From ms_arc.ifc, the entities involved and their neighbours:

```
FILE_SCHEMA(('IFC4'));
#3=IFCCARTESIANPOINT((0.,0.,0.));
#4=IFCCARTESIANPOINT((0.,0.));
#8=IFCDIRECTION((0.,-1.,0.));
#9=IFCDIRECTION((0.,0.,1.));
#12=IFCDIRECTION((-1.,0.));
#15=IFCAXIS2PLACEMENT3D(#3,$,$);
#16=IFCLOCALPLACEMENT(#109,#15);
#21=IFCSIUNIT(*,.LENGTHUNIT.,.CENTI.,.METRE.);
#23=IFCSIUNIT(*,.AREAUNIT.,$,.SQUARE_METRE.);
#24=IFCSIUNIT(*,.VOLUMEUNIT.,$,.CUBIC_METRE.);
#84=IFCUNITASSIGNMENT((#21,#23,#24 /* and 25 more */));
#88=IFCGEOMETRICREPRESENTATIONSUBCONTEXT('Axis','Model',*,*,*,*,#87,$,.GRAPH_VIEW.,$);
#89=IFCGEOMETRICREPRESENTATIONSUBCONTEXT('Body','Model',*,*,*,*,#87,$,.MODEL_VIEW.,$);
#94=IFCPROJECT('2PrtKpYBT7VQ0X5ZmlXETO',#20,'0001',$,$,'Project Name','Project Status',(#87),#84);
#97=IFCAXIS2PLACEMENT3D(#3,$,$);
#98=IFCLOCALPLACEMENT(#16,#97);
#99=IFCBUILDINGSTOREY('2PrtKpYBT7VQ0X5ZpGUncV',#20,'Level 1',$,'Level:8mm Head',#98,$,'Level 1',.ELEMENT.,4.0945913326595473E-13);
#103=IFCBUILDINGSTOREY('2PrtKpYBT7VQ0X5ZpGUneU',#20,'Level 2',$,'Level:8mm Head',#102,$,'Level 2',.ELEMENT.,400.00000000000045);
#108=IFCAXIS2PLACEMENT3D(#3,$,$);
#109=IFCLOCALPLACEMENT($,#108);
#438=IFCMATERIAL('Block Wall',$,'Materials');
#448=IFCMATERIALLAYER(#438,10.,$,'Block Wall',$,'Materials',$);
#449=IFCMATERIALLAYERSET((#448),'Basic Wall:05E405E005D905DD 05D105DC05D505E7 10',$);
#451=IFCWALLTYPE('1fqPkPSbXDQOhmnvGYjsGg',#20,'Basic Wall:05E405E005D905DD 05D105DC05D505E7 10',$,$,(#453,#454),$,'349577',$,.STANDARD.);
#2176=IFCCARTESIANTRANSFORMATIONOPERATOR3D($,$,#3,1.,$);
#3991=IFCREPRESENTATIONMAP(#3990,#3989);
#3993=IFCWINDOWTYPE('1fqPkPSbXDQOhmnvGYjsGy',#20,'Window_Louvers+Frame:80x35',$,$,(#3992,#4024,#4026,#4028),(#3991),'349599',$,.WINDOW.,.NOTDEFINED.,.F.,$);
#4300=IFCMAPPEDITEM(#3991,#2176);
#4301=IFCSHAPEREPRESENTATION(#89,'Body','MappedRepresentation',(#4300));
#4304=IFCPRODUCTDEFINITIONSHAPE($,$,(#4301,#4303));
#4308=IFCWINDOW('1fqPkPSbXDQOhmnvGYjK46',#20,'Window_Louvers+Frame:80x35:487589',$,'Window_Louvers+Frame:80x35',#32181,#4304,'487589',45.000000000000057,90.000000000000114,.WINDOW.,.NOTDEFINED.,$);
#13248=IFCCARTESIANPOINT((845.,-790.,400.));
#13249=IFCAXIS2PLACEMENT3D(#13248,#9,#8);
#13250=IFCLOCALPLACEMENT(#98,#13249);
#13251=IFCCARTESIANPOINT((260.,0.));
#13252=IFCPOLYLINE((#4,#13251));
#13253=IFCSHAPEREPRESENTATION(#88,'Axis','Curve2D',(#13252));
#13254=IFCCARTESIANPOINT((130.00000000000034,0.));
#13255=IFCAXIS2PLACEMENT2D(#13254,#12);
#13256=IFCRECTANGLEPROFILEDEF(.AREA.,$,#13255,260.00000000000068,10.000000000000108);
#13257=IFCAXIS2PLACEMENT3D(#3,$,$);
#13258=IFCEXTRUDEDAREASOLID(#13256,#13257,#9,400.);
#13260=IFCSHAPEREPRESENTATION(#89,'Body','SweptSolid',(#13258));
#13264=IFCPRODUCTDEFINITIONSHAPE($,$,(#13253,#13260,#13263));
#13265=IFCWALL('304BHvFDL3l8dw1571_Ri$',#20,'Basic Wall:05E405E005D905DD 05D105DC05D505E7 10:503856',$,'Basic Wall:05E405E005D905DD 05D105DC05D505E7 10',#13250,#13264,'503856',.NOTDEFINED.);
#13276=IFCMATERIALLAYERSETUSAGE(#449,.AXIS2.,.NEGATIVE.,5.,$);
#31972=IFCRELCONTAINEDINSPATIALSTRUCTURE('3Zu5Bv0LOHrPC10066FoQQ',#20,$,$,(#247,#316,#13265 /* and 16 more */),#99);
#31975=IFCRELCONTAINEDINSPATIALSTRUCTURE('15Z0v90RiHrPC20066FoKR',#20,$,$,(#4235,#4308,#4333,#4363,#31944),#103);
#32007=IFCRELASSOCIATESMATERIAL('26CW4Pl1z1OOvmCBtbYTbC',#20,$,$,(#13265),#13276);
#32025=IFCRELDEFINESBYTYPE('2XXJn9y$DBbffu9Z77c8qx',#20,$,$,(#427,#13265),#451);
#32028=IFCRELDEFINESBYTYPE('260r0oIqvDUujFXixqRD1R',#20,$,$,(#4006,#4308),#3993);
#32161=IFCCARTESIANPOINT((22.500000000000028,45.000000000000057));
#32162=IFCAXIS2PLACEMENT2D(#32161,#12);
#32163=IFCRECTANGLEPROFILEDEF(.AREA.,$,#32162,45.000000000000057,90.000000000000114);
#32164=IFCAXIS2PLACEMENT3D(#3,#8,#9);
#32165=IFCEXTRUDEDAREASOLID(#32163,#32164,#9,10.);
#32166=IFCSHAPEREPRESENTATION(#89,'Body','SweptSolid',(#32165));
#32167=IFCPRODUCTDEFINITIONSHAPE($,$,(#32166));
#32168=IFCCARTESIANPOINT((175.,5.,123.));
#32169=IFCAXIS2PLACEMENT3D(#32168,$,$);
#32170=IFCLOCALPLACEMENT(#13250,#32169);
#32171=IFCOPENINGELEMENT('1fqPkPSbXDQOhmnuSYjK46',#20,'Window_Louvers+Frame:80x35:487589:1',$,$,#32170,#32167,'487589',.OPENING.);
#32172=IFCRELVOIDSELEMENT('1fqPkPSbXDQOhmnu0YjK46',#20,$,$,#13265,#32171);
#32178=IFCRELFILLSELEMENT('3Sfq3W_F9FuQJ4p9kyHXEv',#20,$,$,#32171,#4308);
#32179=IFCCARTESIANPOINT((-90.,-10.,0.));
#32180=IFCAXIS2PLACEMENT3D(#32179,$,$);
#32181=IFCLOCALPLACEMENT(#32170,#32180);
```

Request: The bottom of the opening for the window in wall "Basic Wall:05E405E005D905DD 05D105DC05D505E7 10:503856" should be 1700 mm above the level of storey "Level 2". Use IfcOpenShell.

```python
import numpy as np
import ifcopenshell
import ifcopenshell.api.geometry
import ifcopenshell.geom
import ifcopenshell.util.element
import ifcopenshell.util.placement
import ifcopenshell.util.shape
import ifcopenshell.util.unit

model = ifcopenshell.open("ms_arc.ifc")
unit_scale = ifcopenshell.util.unit.calculate_unit_scale(model)

window = model.by_guid("1fqPkPSbXDQOhmnvGYjK46")
opening = window.FillsVoids[0].RelatingOpeningElement
storey = ifcopenshell.util.element.get_container(window, ifc_class="IfcBuildingStorey")
level = ifcopenshell.util.placement.get_local_placement(storey.ObjectPlacement)[2, 3]

# The opening's origin need not be at the sill, so measure its lowest point.
shape = ifcopenshell.geom.create_shape(ifcopenshell.geom.settings(), opening)
bottom = ifcopenshell.util.shape.get_shape_bottom_elevation(shape, shape.geometry) / unit_scale
dz = level + 1.7 / unit_scale - bottom

shift = np.array([0.0, 0.0, dz])
# The window is placed relative to its opening, so it follows when the opening moves.
matrix = ifcopenshell.util.placement.get_local_placement(opening.ObjectPlacement)
matrix[:3, 3] += shift
ifcopenshell.api.geometry.edit_object_placement(
    model, product=opening, matrix=matrix, is_si=False, should_transform_children=True
)

print(f"moved by {dz * unit_scale:+.3f} m")

model.write("ms_arc_edited.ifc")
```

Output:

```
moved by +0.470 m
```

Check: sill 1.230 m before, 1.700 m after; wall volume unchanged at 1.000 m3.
